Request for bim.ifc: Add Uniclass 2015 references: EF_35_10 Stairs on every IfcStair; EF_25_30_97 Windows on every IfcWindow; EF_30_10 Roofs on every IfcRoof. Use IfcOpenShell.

First a look at what the model holds.

```python
import ifcopenshell

model = ifcopenshell.open("bim.ifc")
print(model.schema)
print("classifications:", [c.Name for c in model.by_type("IfcClassification")])
for ifc_class in ("IfcDoor", "IfcRoof", "IfcStair", "IfcWall", "IfcWindow"):
    print(ifc_class, len(model.by_type(ifc_class)))
```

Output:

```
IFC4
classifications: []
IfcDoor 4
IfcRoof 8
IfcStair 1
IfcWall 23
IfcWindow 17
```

```python
import ifcopenshell
import ifcopenshell.api.classification

model = ifcopenshell.open("bim.ifc")

system = ifcopenshell.api.classification.add_classification(model, classification="Uniclass 2015")

codes = {
    "IfcStair": ("EF_35_10", "Stairs"),
    "IfcWindow": ("EF_25_30_97", "Windows"),
    "IfcRoof": ("EF_30_10", "Roofs"),
}
for ifc_class, (code, name) in codes.items():
    products = model.by_type(ifc_class)
    ifcopenshell.api.classification.add_reference(
        model, products=products, classification=system, identification=code, name=name
    )
    print(code, len(products))

model.write("bim_rev.ifc")
```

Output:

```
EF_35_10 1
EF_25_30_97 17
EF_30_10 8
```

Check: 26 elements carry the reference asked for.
